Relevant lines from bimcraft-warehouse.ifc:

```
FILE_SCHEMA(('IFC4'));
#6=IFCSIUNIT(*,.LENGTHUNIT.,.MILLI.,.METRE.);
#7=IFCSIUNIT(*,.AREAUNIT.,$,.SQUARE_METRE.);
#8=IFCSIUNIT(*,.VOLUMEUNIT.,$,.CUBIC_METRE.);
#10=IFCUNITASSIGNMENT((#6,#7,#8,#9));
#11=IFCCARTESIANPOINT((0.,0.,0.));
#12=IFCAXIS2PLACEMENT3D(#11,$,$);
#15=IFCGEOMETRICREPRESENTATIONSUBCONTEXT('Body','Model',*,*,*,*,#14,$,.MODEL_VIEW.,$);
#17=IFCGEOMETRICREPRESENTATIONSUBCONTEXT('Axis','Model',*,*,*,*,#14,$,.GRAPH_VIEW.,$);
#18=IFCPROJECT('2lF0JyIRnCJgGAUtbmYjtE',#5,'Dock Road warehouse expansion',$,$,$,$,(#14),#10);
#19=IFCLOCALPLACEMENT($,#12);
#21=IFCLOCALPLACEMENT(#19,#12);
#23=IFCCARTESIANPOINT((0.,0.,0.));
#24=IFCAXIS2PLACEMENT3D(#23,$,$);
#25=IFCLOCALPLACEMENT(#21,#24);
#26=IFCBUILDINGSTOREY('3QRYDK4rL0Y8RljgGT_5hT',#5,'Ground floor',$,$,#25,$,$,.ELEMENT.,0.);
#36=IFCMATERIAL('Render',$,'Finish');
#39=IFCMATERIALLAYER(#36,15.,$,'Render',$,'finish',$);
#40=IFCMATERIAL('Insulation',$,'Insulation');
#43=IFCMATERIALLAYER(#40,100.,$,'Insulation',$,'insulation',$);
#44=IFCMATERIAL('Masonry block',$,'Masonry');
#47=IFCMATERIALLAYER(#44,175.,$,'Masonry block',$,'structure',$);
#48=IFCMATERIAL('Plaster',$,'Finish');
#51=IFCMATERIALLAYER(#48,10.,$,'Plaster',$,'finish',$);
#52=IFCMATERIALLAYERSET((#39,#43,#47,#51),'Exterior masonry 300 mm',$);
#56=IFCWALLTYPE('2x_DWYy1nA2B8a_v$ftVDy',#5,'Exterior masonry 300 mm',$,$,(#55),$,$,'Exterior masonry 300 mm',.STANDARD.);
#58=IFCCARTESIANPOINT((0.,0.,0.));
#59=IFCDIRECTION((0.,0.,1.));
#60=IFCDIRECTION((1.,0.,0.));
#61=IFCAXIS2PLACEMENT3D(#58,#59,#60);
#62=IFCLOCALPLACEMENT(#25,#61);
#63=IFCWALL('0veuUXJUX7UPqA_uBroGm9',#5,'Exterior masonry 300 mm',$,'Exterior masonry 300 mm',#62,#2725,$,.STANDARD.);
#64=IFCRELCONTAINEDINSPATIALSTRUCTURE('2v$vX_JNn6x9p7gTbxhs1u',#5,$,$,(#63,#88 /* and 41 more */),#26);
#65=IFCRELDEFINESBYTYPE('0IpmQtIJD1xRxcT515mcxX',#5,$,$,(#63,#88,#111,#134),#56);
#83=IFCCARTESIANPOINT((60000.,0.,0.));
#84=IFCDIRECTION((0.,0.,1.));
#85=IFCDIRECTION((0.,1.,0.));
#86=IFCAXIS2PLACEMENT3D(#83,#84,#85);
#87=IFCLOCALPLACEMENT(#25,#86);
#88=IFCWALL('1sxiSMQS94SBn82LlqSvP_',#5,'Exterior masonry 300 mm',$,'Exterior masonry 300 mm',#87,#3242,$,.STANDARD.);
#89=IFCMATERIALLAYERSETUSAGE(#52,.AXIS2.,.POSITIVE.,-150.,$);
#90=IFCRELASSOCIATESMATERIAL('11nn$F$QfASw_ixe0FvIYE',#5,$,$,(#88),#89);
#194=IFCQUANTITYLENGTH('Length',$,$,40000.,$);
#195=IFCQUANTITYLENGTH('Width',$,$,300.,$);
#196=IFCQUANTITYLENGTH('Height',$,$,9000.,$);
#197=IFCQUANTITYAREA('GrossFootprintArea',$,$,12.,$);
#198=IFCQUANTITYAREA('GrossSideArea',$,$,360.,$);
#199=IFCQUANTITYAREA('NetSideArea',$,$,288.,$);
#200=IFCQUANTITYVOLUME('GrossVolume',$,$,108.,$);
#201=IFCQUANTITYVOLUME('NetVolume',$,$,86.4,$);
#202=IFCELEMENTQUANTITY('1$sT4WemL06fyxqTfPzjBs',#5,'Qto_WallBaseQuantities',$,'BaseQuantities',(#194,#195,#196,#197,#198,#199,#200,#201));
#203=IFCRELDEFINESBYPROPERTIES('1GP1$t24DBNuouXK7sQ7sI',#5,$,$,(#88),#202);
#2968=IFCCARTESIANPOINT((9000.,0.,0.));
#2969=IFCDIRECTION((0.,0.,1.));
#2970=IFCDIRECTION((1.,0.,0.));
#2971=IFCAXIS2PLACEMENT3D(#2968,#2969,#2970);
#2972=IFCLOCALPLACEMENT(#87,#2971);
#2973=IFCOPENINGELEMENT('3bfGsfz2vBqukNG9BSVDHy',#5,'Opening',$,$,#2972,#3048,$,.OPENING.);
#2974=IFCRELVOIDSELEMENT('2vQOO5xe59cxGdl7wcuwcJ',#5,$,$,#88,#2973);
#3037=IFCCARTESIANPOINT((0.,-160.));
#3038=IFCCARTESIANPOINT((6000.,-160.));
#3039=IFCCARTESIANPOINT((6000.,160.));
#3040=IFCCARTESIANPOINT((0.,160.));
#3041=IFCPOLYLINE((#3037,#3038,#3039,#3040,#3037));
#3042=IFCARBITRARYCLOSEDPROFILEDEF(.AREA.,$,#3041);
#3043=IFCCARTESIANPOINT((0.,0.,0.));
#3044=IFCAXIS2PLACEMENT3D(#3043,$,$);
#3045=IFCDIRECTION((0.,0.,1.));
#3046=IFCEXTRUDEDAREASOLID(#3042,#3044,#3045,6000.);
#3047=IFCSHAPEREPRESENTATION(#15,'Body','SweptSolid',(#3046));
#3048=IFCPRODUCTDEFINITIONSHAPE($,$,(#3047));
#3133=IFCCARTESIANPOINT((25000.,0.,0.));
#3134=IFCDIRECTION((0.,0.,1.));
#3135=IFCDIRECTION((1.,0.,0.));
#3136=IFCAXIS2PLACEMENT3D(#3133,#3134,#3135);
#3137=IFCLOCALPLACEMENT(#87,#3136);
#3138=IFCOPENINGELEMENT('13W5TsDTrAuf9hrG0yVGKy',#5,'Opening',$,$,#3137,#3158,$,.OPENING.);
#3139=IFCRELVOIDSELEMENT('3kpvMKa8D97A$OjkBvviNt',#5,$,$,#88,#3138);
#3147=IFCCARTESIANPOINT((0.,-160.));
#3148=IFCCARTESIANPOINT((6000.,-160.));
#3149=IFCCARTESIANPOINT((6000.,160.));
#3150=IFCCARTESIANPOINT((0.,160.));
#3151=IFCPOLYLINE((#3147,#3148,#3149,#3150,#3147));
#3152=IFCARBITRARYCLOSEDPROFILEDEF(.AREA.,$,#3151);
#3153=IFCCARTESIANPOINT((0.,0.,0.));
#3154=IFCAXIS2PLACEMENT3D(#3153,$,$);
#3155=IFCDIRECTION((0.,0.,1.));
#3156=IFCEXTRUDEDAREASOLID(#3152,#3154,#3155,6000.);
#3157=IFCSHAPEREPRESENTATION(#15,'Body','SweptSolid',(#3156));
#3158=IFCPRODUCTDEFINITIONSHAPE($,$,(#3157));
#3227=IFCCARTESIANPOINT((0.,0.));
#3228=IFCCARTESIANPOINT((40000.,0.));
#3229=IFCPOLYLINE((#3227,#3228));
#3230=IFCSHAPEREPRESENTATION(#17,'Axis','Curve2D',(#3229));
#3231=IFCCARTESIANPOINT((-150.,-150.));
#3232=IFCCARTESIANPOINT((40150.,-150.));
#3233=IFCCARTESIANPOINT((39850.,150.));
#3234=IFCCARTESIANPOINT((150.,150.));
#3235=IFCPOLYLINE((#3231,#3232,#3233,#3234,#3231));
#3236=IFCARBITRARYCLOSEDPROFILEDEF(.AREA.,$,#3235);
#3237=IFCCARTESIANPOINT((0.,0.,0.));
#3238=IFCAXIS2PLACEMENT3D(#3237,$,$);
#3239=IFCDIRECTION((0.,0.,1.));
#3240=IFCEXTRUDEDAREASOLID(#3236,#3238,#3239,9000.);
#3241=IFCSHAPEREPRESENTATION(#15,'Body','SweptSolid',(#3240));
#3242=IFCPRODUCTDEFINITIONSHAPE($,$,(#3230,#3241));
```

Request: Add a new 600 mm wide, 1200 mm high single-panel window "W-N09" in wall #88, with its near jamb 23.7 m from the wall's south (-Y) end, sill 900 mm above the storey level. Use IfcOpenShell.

```python
import numpy as np
import ifcopenshell
import ifcopenshell.api.feature
import ifcopenshell.api.geometry
import ifcopenshell.api.pset
import ifcopenshell.api.root
import ifcopenshell.api.spatial
import ifcopenshell.geom
import ifcopenshell.util.element
import ifcopenshell.util.placement
import ifcopenshell.util.representation
import ifcopenshell.util.shape
import ifcopenshell.util.unit

model = ifcopenshell.open("bimcraft-warehouse.ifc")
unit_scale = ifcopenshell.util.unit.calculate_unit_scale(model)
area_scale = ifcopenshell.util.unit.calculate_unit_scale(model, "AREAUNIT")
volume_scale = ifcopenshell.util.unit.calculate_unit_scale(model, "VOLUMEUNIT")
settings = ifcopenshell.geom.settings()


def volume(element):
    """Net volume in cubic metres, openings subtracted."""
    shape = ifcopenshell.geom.create_shape(settings, element)
    return ifcopenshell.util.shape.get_volume(shape.geometry)


wall = model.by_id(88)
storey = ifcopenshell.util.element.get_container(wall, ifc_class="IfcBuildingStorey")
context = ifcopenshell.util.representation.get_context(model, "Model", "Body", "MODEL_VIEW")
before = volume(wall)

width, height, from_end, sill = 0.6, 1.2, 23.7, 0.9  # metres

# The wall runs along its own X axis, and the end named is its -X end.
wall_shape = ifcopenshell.geom.create_shape(settings, wall)
x, y, z = ifcopenshell.util.shape.get_vertices(wall_shape.geometry).T
start = x.min() + from_end
face, thickness = float(y.min()), float(y.max() - y.min())
wall_matrix = ifcopenshell.util.placement.get_local_placement(wall.ObjectPlacement)
level = ifcopenshell.util.placement.get_local_placement(storey.ObjectPlacement)[2, 3]


def in_wall(x, y):
    """Placement at x, y metres in the wall's axes, at sill height."""
    matrix = wall_matrix.copy()
    matrix[:, 3] = wall_matrix @ np.array([x / unit_scale, y / unit_scale, 0.0, 1.0])
    matrix[2, 3] = level + sill / unit_scale
    return matrix


# Opening: a box that overshoots both wall faces by 50 mm.
opening = ifcopenshell.api.root.create_entity(model, ifc_class="IfcOpeningElement", predefined_type="OPENING")
box = ifcopenshell.api.geometry.add_wall_representation(
    model, context=context, length=width, height=height, thickness=thickness + 0.1
)
ifcopenshell.api.geometry.assign_representation(model, product=opening, representation=box)
ifcopenshell.api.geometry.edit_object_placement(model, product=opening, matrix=in_wall(start, face - 0.05), is_si=False)
ifcopenshell.api.feature.add_feature(model, feature=opening, element=wall)

window = ifcopenshell.api.root.create_entity(model, ifc_class="IfcWindow", name="W-N09", predefined_type="WINDOW")
window.OverallWidth, window.OverallHeight = width / unit_scale, height / unit_scale
window.PartitioningType = "SINGLE_PANEL"
body = ifcopenshell.api.geometry.add_window_representation(
    model,
    context=context,
    overall_width=window.OverallWidth,
    overall_height=window.OverallHeight,
    partition_type="SINGLE_PANEL",
)
ifcopenshell.api.geometry.assign_representation(model, product=window, representation=body)
ifcopenshell.api.spatial.assign_container(model, products=[window], relating_structure=storey)
ifcopenshell.api.feature.add_filling(model, opening=opening, element=window)

# Centre the window in the wall's thickness.
ifcopenshell.api.geometry.edit_object_placement(model, product=window, matrix=in_wall(start, face), is_si=False)
window_shape = ifcopenshell.geom.create_shape(settings, window)
depth = ifcopenshell.util.shape.get_vertices(window_shape.geometry)[:, 1]
offset = face + thickness / 2 - (depth.min() + depth.max()) / 2
ifcopenshell.api.geometry.edit_object_placement(model, product=window, matrix=in_wall(start, offset), is_si=False)

after = volume(wall)

# Update the wall's stored quantities.
qto = model.by_id(ifcopenshell.util.element.get_pset(wall, "Qto_WallBaseQuantities", should_inherit=False)["id"])
ifcopenshell.api.pset.edit_qto(model, qto=qto, properties={
    "NetSideArea": after / thickness / area_scale,
    "NetVolume": after / volume_scale,
})

print(f"wall volume {before:.3f} -> {after:.3f} m3")

model.write("bimcraft-warehouse_updated.ifc")
```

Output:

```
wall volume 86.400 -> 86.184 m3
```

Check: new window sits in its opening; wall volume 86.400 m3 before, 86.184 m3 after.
